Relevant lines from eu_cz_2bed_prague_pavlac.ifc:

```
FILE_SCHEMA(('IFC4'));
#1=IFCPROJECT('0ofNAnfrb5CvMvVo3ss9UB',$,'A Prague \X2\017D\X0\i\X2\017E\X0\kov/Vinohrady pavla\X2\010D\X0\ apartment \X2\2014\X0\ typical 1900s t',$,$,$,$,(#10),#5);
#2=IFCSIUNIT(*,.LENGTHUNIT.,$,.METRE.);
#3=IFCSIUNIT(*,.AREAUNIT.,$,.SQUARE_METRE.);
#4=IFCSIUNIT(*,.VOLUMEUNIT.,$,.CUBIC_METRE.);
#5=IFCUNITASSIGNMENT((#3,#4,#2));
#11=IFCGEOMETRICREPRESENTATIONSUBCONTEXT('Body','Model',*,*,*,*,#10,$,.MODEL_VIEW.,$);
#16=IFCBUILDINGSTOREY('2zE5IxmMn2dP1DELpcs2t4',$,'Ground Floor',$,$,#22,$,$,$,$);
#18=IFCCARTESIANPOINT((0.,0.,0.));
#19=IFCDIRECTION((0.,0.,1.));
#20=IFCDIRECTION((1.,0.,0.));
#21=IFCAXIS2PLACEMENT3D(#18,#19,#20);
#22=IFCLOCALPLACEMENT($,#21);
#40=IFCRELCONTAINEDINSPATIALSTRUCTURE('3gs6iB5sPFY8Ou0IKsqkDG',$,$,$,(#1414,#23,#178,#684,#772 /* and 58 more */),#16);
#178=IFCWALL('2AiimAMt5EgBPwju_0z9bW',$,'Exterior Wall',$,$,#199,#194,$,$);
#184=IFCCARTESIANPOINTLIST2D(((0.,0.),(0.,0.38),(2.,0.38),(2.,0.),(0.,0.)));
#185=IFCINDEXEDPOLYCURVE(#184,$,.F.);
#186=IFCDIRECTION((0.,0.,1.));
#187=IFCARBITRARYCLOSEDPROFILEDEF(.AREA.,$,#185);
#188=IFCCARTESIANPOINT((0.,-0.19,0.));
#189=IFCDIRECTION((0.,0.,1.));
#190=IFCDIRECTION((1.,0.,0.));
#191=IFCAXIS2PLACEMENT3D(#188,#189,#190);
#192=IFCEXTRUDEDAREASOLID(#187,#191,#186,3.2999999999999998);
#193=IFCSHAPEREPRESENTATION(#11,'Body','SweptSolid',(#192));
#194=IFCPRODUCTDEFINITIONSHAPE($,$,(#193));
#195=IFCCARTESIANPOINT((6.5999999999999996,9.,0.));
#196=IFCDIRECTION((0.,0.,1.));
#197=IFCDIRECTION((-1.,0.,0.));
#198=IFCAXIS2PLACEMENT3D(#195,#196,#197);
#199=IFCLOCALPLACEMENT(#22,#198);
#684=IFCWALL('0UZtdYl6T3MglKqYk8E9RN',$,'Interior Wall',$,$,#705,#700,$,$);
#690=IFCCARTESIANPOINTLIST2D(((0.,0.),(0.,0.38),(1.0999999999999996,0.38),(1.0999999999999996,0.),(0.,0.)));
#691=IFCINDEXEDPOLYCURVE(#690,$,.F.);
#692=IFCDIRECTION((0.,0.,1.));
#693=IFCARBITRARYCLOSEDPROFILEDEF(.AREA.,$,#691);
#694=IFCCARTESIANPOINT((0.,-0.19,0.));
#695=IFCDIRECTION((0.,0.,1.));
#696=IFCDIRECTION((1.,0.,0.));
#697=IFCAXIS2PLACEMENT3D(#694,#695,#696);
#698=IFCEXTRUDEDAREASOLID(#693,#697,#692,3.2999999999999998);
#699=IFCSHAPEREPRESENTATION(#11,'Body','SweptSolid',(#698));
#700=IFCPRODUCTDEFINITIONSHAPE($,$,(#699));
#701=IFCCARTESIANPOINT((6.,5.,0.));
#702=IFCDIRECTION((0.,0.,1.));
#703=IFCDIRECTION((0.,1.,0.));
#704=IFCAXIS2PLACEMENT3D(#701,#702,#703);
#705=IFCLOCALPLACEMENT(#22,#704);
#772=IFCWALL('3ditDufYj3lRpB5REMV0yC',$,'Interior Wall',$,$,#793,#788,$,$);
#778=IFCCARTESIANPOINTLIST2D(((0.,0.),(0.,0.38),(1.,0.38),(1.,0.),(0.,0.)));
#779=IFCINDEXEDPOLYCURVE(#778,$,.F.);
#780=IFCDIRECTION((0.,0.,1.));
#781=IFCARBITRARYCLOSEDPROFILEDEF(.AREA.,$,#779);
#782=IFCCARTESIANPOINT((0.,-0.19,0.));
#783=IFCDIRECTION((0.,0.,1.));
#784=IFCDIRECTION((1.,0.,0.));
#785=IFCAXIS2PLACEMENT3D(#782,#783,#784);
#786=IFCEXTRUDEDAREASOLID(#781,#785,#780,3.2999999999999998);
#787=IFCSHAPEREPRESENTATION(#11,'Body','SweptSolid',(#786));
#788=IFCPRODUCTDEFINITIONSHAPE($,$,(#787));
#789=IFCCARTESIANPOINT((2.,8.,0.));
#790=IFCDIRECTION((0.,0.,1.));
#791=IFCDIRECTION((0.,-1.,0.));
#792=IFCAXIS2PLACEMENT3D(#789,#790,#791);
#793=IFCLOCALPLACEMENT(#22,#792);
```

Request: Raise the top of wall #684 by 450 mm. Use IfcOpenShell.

```python
import ifcopenshell
import ifcopenshell.geom
import ifcopenshell.util.representation
import ifcopenshell.util.shape

model = ifcopenshell.open("eu_cz_2bed_prague_pavlac.ifc")
settings = ifcopenshell.geom.settings()


def volume(element):
    """Net volume in cubic metres, openings subtracted."""
    shape = ifcopenshell.geom.create_shape(settings, element)
    return ifcopenshell.util.shape.get_volume(shape.geometry)


wall = model.by_guid("0UZtdYl6T3MglKqYk8E9RN")
before = volume(wall)

body = ifcopenshell.util.representation.get_representation(wall, "Model", "Body")
solid = body.Items[0]
old_height = solid.Depth
solid.Depth += 0.45
after = volume(wall)

print(f"height {old_height:g} -> {solid.Depth:g}, volume {before:.3f} -> {after:.3f} m3")

model.write("eu_cz_2bed_prague_pavlac_edited.ifc")
```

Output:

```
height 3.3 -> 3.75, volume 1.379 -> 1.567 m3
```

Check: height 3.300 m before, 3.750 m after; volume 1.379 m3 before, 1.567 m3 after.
